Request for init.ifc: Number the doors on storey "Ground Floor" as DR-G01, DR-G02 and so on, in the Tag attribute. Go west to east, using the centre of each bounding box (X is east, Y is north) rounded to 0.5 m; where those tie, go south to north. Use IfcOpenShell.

First a look at what the model holds.

```python
import ifcopenshell
import ifcopenshell.util.element
import ifcopenshell.util.placement

model = ifcopenshell.open("init.ifc")
print(model.schema)
storey = next(s for s in model.by_type("IfcBuildingStorey") if s.Name == "Ground Floor")
doors = [e for e in ifcopenshell.util.element.get_decomposition(storey) if e.is_a("IfcDoor")]
for e in sorted(doors, key=lambda e: e.id()):
    origin = ifcopenshell.util.placement.get_local_placement(e.ObjectPlacement)[:3, 3]
    print(e.id(), e.Tag, e.Name, origin.round(2) + 0.0, sep=" | ")
```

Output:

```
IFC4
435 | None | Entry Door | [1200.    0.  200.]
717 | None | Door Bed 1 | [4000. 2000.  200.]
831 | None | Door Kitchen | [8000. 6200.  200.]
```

```python
import ifcopenshell
import ifcopenshell.geom
import ifcopenshell.util.element
import ifcopenshell.util.shape

model = ifcopenshell.open("init.ifc")
settings = ifcopenshell.geom.settings()
settings.set("use-world-coords", True)


def centre(element):
    shape = ifcopenshell.geom.create_shape(settings, element)
    return ifcopenshell.util.shape.get_bbox_centroid(shape.geometry)


storey = next(s for s in model.by_type("IfcBuildingStorey") if s.Name == "Ground Floor")
doors = [e for e in ifcopenshell.util.element.get_decomposition(storey) if e.is_a("IfcDoor")]

# Insertion points can sit at a corner or the storey origin, so sort by the geometry (in metres).
centres = {e: centre(e) for e in doors}
doors.sort(key=lambda e: (round(centres[e][0] / 0.5), centres[e][1]))

for i, e in enumerate(doors, start=1):
    number = f"DR-G{i:02d}"
    e.Tag = number
    print(e.id(), number)

model.write("init_rev.ifc")
```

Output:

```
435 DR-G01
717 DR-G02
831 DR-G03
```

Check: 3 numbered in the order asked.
